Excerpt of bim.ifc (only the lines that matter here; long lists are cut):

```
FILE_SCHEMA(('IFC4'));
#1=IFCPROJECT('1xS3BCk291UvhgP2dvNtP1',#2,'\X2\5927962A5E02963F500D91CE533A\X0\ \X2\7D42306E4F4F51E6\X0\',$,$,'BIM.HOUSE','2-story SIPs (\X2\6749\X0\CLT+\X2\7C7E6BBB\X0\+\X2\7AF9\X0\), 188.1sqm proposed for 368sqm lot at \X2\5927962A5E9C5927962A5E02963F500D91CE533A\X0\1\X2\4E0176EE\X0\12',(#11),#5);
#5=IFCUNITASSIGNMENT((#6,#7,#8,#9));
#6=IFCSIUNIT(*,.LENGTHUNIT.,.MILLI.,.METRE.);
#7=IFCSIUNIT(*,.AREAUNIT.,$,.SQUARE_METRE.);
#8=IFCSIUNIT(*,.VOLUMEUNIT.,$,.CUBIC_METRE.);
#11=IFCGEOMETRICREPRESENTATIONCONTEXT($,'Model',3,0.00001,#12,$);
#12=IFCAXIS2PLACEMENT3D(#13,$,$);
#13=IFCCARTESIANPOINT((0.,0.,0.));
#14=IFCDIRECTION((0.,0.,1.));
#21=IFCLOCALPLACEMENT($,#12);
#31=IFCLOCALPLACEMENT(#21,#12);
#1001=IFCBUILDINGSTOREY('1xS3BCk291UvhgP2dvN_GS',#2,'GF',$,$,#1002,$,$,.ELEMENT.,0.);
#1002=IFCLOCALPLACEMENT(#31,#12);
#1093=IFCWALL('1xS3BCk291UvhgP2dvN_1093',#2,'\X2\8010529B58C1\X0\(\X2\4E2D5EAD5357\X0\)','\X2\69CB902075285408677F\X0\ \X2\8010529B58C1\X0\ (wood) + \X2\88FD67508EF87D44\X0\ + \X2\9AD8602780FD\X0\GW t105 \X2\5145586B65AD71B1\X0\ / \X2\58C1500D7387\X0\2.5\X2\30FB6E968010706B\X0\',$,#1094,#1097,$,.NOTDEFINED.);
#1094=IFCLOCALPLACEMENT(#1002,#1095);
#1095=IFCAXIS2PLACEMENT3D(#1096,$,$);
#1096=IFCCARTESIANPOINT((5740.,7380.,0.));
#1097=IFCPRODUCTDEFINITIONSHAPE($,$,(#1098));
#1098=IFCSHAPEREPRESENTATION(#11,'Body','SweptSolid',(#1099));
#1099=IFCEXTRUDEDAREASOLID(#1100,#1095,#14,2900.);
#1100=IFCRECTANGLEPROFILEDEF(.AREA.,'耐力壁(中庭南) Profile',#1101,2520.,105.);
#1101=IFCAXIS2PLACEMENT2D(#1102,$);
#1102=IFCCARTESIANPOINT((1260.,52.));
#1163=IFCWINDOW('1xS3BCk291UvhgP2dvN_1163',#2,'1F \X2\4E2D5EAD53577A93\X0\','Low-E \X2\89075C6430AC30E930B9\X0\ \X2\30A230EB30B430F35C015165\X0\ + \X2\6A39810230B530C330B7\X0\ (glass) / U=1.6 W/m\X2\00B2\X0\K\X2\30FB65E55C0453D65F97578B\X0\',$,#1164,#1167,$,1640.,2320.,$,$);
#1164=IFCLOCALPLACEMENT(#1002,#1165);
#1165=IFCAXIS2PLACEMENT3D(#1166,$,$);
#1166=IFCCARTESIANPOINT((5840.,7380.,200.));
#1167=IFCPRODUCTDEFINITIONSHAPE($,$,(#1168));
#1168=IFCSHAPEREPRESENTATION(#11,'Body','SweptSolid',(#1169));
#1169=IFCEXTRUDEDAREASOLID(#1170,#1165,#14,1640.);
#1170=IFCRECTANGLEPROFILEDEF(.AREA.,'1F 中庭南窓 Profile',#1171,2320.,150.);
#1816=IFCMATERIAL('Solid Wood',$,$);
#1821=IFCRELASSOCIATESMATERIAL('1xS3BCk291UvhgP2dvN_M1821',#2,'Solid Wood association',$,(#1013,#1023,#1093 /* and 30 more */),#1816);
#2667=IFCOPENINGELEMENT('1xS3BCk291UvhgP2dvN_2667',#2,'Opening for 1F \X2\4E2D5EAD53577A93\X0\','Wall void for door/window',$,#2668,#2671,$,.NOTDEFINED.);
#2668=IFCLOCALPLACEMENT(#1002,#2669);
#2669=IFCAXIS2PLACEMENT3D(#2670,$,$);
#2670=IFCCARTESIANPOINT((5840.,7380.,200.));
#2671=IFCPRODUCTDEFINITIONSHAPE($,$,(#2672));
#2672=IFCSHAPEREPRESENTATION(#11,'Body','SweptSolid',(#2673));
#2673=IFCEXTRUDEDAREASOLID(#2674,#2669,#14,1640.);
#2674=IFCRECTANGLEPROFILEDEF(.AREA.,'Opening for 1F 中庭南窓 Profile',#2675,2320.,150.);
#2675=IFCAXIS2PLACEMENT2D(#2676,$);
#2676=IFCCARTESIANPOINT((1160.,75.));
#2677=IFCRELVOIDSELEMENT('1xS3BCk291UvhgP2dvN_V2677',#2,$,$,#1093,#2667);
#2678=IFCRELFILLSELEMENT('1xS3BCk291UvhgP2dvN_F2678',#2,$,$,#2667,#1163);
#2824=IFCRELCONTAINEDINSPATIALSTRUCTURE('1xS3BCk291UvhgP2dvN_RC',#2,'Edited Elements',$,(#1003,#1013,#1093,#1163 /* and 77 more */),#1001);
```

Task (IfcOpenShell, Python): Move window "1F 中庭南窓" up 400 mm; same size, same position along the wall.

```python
import numpy as np
import ifcopenshell
import ifcopenshell.api.geometry
import ifcopenshell.util.placement
import ifcopenshell.util.unit

model = ifcopenshell.open("bim.ifc")
unit_scale = ifcopenshell.util.unit.calculate_unit_scale(model)

window = model.by_guid("1xS3BCk291UvhgP2dvN_1163")
opening = window.FillsVoids[0].RelatingOpeningElement
dz = 400.0

shift = np.array([0.0, 0.0, dz])
# The window is not placed relative to its opening, so move both.
for product in (opening, window):
    matrix = ifcopenshell.util.placement.get_local_placement(product.ObjectPlacement)
    matrix[:3, 3] += shift
    ifcopenshell.api.geometry.edit_object_placement(model, product=product, matrix=matrix, is_si=False)

print(f"moved by {dz * unit_scale:+.3f} m")

model.write("bim_v2.ifc")
```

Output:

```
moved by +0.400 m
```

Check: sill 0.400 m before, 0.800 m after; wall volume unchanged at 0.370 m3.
